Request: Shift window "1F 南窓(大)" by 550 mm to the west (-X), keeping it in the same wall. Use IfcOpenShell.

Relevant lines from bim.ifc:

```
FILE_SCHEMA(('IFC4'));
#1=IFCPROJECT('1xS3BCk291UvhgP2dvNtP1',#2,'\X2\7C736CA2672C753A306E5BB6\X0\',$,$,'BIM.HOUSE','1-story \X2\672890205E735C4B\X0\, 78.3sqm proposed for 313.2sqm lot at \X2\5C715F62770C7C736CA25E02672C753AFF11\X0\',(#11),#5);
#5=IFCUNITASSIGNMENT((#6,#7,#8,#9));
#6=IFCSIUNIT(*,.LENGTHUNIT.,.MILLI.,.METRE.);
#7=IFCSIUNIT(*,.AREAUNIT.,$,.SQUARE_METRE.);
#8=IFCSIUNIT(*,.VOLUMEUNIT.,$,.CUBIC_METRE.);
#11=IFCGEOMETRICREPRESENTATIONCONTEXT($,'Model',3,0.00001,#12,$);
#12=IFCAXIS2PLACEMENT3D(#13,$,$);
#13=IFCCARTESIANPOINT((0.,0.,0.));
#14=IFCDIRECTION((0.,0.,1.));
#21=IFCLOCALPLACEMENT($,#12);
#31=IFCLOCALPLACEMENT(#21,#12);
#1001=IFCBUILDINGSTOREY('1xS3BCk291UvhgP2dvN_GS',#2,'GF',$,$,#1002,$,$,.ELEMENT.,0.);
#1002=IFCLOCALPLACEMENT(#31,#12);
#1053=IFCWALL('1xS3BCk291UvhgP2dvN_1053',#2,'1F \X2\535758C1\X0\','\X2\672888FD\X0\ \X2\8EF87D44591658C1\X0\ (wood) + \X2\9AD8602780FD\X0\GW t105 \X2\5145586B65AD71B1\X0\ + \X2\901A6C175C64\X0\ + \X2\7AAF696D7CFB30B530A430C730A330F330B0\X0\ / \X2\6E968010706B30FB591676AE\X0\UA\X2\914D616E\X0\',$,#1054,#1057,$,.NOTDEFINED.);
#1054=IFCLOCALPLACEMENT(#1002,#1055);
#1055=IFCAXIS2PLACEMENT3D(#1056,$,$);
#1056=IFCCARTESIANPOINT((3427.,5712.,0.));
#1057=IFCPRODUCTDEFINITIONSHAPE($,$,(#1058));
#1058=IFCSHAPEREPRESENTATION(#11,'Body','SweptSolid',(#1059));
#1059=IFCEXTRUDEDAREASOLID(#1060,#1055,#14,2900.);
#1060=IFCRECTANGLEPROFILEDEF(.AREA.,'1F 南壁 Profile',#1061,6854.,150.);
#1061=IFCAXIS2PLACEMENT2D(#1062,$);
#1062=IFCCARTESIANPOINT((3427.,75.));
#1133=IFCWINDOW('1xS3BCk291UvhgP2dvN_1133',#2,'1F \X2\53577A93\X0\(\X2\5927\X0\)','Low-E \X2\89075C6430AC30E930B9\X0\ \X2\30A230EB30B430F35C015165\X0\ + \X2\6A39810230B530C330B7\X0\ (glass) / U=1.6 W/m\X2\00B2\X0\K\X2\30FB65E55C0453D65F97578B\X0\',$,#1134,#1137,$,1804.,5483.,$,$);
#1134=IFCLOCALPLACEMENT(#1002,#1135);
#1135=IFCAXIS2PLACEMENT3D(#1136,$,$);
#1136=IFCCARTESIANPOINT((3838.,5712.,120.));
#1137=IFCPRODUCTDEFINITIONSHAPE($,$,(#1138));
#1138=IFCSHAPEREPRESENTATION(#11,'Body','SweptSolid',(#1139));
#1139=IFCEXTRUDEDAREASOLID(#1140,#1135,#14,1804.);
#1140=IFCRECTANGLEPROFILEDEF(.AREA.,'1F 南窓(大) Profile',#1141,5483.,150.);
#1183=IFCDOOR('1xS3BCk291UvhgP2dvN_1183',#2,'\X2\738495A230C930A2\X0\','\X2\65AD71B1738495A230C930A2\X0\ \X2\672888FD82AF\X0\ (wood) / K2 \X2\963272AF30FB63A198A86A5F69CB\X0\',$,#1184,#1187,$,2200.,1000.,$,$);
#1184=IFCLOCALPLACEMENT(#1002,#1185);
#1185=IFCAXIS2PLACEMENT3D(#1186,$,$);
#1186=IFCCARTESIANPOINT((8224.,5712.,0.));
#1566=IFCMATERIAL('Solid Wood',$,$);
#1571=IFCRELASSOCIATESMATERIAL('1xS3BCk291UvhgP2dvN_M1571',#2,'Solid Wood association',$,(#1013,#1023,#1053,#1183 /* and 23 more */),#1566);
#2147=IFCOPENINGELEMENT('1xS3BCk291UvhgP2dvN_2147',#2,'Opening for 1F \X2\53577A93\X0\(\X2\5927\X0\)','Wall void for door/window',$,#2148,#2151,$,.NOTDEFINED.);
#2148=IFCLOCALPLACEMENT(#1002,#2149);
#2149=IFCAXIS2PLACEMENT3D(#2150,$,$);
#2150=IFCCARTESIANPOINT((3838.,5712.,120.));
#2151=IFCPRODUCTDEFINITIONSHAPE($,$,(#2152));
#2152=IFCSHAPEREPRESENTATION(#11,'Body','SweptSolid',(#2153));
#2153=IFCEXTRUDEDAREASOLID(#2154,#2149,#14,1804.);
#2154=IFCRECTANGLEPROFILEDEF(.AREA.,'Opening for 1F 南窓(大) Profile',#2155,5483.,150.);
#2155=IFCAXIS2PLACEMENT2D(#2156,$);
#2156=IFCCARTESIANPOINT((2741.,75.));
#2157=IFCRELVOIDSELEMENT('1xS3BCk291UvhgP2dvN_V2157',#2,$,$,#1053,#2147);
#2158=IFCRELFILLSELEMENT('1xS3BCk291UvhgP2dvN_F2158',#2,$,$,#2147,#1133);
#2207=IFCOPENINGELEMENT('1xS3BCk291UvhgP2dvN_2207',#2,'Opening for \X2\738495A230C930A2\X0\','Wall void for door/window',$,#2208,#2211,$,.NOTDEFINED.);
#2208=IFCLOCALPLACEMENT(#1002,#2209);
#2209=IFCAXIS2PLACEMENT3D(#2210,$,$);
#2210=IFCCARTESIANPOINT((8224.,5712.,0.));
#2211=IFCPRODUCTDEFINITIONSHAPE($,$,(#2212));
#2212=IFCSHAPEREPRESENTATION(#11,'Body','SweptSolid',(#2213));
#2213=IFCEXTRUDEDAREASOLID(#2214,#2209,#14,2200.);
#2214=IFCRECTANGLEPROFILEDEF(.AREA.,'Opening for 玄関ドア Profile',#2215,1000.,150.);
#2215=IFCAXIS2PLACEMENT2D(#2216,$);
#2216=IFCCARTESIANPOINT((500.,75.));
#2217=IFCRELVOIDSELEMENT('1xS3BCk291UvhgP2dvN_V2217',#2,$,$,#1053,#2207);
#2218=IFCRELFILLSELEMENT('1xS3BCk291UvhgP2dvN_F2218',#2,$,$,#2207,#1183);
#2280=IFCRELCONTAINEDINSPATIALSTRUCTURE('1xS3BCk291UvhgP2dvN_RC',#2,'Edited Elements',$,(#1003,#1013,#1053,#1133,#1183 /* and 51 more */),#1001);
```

```python
import ifcopenshell
import ifcopenshell.api.geometry
import ifcopenshell.util.placement
import ifcopenshell.util.unit

model = ifcopenshell.open("bim.ifc")
unit_scale = ifcopenshell.util.unit.calculate_unit_scale(model)

window = model.by_guid("1xS3BCk291UvhgP2dvN_1133")
opening = window.FillsVoids[0].RelatingOpeningElement
wall = opening.VoidsElements[0].RelatingBuildingElement

wall_matrix = ifcopenshell.util.placement.get_local_placement(wall.ObjectPlacement)
shift = wall_matrix[:3, 0] * -0.55 / unit_scale
before = ifcopenshell.util.placement.get_local_placement(window.ObjectPlacement)[:3, 3].copy()

# The window is not placed relative to its opening, so move both.
for product in (opening, window):
    matrix = ifcopenshell.util.placement.get_local_placement(product.ObjectPlacement)
    matrix[:3, 3] += shift
    ifcopenshell.api.geometry.edit_object_placement(model, product=product, matrix=matrix, is_si=False)

after = ifcopenshell.util.placement.get_local_placement(window.ObjectPlacement)[:3, 3]
print("window moved by", (after - before).round(3) + 0.0)

model.write("bim-out.ifc")
```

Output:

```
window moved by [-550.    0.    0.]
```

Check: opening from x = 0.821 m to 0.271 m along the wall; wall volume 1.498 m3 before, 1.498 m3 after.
